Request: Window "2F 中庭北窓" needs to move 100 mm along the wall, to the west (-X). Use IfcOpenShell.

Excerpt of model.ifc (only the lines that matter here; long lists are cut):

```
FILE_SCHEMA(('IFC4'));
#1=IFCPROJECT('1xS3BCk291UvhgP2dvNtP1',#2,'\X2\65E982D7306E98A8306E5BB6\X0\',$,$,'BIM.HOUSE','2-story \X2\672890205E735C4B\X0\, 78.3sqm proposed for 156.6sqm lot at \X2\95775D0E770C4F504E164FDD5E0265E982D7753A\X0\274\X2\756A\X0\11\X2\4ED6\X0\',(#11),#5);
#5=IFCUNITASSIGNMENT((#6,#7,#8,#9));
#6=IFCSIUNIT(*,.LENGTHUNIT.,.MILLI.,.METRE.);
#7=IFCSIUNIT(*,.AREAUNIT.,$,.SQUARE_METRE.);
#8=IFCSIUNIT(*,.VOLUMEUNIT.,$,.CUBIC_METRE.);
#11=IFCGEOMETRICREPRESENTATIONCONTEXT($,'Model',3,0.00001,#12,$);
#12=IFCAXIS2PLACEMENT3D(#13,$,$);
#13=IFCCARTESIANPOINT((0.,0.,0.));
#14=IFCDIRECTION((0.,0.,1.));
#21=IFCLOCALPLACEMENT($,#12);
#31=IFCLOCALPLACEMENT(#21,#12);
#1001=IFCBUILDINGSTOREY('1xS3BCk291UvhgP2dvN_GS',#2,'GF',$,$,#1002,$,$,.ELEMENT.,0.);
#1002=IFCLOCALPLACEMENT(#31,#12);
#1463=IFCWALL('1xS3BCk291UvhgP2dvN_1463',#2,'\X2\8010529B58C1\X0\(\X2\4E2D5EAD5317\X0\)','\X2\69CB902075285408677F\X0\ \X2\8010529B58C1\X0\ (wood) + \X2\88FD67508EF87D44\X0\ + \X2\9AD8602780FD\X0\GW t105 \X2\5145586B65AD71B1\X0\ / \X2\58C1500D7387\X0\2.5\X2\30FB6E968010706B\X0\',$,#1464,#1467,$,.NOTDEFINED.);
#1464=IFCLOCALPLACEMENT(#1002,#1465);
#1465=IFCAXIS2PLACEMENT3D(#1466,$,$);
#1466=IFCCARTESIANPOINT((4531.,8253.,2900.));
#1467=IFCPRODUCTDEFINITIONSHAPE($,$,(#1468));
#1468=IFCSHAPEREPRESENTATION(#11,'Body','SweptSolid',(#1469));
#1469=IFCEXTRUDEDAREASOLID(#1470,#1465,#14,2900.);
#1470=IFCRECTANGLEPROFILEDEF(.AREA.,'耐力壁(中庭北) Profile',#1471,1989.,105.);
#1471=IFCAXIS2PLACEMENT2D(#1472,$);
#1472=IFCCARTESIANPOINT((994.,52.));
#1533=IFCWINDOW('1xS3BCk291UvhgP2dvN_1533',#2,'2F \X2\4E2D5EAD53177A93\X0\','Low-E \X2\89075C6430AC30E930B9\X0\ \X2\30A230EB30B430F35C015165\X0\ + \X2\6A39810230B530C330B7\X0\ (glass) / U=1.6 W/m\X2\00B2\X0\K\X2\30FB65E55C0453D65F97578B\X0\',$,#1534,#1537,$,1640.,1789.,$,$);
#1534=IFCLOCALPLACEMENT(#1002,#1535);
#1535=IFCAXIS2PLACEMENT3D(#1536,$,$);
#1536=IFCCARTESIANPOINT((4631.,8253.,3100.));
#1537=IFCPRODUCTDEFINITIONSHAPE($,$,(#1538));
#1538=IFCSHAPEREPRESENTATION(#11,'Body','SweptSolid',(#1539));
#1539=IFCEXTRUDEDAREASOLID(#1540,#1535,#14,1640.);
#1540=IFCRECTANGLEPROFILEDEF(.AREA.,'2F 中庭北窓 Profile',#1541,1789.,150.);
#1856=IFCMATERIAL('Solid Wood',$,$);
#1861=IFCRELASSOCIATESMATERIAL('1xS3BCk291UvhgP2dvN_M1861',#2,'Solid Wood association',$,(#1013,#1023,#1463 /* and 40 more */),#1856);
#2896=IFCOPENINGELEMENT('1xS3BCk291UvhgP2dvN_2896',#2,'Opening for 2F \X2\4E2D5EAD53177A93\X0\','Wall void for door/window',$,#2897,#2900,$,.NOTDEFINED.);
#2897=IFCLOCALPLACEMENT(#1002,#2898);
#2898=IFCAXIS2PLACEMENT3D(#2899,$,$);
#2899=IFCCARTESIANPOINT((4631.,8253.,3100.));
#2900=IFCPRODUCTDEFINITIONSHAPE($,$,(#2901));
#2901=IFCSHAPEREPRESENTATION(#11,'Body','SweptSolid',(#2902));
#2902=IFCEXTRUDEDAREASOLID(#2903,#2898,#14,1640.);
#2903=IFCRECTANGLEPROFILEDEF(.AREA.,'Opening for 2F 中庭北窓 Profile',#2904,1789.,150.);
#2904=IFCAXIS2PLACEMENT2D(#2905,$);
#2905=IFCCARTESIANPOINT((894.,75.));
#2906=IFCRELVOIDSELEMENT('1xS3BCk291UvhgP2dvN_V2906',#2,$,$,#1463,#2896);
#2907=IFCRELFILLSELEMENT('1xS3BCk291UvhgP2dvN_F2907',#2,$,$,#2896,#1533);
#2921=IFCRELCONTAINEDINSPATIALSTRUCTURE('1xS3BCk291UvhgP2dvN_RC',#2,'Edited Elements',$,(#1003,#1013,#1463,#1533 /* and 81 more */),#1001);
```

```python
import ifcopenshell
import ifcopenshell.api.geometry
import ifcopenshell.util.placement
import ifcopenshell.util.unit

model = ifcopenshell.open("model.ifc")
unit_scale = ifcopenshell.util.unit.calculate_unit_scale(model)

window = model.by_guid("1xS3BCk291UvhgP2dvN_1533")
opening = window.FillsVoids[0].RelatingOpeningElement
wall = opening.VoidsElements[0].RelatingBuildingElement

wall_matrix = ifcopenshell.util.placement.get_local_placement(wall.ObjectPlacement)
shift = wall_matrix[:3, 0] * -0.1 / unit_scale
before = ifcopenshell.util.placement.get_local_placement(window.ObjectPlacement)[:3, 3].copy()

# The window is not placed relative to its opening, so move both.
for product in (opening, window):
    matrix = ifcopenshell.util.placement.get_local_placement(product.ObjectPlacement)
    matrix[:3, 3] += shift
    ifcopenshell.api.geometry.edit_object_placement(model, product=product, matrix=matrix, is_si=False)

after = ifcopenshell.util.placement.get_local_placement(window.ObjectPlacement)[:3, 3]
print("window moved by", (after - before).round(3) + 0.0)

model.write("model-out.ifc")
```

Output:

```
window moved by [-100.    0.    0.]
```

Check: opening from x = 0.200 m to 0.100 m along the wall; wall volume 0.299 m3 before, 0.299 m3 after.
